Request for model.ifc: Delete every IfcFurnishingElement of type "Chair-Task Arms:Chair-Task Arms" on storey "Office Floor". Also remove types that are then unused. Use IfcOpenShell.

First a look at what the model holds.

```python
import ifcopenshell
import ifcopenshell.util.element

model = ifcopenshell.open("model.ifc")
print(model.schema)
storey = next(s for s in model.by_type("IfcBuildingStorey") if s.Name == "Office Floor")
furniture = [e for e in ifcopenshell.util.element.get_decomposition(storey) if e.is_a("IfcFurnishingElement")]
seen = {}
for e in furniture:
    element_type = ifcopenshell.util.element.get_type(e)
    name = element_type.Name if element_type not in (None, e) else None
    seen[name] = seen.get(name, 0) + 1
for name, count in sorted(seen.items(), key=str):
    print(count, "x", name)
```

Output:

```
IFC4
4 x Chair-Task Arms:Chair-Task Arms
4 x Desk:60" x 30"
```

```python
import ifcopenshell
import ifcopenshell.api.root
import ifcopenshell.util.element

model = ifcopenshell.open("model.ifc")

storey = next(s for s in model.by_type("IfcBuildingStorey") if s.Name == "Office Floor")
furniture = [e for e in ifcopenshell.util.element.get_decomposition(storey) if e.is_a("IfcFurnishingElement")]
targets = [e for e in furniture if (t := ifcopenshell.util.element.get_type(e)) not in (None, e) and t.Name == "Chair-Task Arms:Chair-Task Arms"]
types = {ifcopenshell.util.element.get_type(e) for e in targets} - {None, *targets}

for e in targets:
    ifcopenshell.api.root.remove_product(model, product=e)
print(len(targets), "removed")

unused = [t for t in types if not ifcopenshell.util.element.get_types(t)]
for t in unused:
    ifcopenshell.api.root.remove_product(model, product=t)
print(len(unused), "unused types removed")

model.write("model_rev.ifc")
```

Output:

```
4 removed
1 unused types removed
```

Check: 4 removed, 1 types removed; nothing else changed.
